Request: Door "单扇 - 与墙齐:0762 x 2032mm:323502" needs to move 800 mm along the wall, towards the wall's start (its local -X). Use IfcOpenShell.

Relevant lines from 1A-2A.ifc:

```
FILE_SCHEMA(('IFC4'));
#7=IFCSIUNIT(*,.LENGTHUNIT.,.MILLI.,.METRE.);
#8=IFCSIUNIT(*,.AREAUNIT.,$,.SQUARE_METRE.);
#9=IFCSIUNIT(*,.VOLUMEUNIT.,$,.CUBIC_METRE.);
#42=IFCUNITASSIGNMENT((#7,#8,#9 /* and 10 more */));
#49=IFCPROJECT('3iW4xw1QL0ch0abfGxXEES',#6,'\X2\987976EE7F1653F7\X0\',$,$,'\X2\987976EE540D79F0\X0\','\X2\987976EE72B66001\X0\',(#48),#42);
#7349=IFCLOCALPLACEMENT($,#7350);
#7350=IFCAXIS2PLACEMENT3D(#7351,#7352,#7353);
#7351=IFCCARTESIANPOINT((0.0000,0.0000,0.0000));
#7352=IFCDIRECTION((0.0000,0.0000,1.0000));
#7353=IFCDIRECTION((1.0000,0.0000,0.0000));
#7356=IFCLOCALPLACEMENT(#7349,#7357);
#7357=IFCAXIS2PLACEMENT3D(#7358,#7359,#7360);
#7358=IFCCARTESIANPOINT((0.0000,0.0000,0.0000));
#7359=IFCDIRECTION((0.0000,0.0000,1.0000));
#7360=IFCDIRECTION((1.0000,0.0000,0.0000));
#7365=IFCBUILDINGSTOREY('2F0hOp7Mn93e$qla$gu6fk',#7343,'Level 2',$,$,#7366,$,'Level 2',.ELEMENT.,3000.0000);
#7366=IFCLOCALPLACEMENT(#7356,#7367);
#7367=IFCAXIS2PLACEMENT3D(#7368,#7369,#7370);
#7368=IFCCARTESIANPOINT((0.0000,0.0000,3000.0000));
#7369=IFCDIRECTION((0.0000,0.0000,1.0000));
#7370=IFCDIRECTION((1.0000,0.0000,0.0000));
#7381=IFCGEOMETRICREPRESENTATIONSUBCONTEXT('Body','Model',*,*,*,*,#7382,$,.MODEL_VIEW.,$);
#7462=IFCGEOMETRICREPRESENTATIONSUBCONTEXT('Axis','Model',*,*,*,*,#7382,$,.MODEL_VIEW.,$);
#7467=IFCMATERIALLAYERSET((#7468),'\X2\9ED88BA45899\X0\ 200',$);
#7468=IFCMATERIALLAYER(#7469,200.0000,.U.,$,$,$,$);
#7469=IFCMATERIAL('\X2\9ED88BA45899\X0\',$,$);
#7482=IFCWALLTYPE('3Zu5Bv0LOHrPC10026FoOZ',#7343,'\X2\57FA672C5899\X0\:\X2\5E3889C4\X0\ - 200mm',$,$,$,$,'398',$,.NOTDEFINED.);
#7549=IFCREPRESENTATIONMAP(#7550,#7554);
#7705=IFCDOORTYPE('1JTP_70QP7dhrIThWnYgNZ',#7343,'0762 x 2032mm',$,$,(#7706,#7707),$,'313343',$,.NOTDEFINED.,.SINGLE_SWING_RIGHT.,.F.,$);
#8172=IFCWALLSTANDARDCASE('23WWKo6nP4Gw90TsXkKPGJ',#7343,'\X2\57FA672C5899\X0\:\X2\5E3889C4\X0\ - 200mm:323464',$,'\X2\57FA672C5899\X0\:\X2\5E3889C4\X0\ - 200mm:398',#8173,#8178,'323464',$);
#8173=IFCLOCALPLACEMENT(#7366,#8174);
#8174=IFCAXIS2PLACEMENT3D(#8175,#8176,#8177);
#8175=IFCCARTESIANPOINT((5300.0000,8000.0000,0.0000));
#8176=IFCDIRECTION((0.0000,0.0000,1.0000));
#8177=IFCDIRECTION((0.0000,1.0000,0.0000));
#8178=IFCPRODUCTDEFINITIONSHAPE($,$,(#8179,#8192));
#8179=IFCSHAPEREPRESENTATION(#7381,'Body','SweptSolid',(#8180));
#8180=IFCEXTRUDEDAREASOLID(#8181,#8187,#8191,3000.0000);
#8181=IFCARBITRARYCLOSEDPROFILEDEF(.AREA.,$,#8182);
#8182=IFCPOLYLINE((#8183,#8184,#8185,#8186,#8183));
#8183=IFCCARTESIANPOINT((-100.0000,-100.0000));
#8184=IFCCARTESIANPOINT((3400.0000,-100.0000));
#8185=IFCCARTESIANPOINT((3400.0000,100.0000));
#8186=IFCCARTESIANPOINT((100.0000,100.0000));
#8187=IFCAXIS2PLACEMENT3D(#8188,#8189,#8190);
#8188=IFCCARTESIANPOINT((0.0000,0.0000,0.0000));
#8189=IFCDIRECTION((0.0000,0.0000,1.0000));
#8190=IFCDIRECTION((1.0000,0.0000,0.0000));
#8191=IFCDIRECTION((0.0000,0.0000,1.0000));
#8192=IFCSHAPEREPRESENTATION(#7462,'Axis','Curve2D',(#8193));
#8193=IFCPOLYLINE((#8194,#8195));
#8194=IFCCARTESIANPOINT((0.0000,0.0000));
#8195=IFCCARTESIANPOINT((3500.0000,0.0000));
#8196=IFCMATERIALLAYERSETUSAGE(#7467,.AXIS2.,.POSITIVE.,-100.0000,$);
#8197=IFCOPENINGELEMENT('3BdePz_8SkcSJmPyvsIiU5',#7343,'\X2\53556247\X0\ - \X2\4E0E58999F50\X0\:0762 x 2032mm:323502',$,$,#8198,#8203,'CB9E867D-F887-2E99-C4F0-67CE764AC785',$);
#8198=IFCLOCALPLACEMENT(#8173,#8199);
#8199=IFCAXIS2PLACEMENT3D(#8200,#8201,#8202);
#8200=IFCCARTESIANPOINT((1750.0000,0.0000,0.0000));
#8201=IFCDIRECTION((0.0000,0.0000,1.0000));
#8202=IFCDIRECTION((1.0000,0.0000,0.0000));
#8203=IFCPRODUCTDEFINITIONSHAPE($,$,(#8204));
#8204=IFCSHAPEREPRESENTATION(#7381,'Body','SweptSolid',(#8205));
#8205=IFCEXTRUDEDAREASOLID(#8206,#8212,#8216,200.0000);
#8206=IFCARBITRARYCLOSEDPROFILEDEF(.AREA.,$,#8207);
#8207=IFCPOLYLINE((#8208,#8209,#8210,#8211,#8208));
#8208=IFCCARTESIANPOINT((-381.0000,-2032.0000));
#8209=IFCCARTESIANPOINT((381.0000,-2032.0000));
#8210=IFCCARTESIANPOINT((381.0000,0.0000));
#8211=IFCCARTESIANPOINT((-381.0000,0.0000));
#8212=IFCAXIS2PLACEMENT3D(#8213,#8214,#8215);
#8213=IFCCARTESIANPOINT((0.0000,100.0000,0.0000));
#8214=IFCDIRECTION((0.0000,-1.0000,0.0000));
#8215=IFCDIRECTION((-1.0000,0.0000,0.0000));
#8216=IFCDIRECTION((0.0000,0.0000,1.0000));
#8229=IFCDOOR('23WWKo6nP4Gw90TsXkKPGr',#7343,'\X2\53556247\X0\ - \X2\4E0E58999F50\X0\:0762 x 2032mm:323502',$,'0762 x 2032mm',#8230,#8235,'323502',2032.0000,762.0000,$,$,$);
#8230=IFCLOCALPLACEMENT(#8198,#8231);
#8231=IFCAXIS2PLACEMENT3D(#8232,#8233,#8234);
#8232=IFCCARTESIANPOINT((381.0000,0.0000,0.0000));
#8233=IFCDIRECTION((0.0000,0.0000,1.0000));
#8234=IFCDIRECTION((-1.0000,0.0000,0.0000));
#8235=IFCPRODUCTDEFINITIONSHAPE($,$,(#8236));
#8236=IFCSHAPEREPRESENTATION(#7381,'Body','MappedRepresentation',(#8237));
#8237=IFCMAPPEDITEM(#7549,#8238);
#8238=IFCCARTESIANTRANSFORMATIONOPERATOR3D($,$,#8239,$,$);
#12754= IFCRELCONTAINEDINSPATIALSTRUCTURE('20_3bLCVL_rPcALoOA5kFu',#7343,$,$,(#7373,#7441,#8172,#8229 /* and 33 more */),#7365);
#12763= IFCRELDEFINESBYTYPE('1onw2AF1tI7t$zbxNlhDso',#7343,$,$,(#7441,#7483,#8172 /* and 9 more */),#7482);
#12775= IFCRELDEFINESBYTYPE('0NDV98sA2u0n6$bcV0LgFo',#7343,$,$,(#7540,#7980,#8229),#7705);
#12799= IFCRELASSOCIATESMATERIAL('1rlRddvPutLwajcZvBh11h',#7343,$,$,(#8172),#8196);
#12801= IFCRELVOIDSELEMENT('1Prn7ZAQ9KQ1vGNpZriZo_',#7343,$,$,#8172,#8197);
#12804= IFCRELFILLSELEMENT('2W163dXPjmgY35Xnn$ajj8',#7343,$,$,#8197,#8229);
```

```python
import ifcopenshell
import ifcopenshell.api.geometry
import ifcopenshell.util.placement
import ifcopenshell.util.unit

model = ifcopenshell.open("1A-2A.ifc")
unit_scale = ifcopenshell.util.unit.calculate_unit_scale(model)

door = model.by_guid("23WWKo6nP4Gw90TsXkKPGr")
opening = door.FillsVoids[0].RelatingOpeningElement
wall = opening.VoidsElements[0].RelatingBuildingElement

wall_matrix = ifcopenshell.util.placement.get_local_placement(wall.ObjectPlacement)
shift = wall_matrix[:3, 0] * -0.8 / unit_scale
before = ifcopenshell.util.placement.get_local_placement(door.ObjectPlacement)[:3, 3].copy()

# The door is placed relative to its opening, so it follows when the opening moves.
matrix = ifcopenshell.util.placement.get_local_placement(opening.ObjectPlacement)
matrix[:3, 3] += shift
ifcopenshell.api.geometry.edit_object_placement(
    model, product=opening, matrix=matrix, is_si=False, should_transform_children=True
)

after = ifcopenshell.util.placement.get_local_placement(door.ObjectPlacement)[:3, 3]
print("door moved by", (after - before).round(3) + 0.0)

model.write("1A-2A_updated.ifc")
```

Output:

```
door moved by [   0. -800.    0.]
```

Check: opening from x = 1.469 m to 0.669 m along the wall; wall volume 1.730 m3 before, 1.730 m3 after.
